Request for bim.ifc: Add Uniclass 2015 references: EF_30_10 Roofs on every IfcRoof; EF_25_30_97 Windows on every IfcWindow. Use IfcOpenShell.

First a look at what the model holds.

```python
import ifcopenshell

model = ifcopenshell.open("bim.ifc")
print(model.schema)
print("classifications:", [c.Name for c in model.by_type("IfcClassification")])
for ifc_class in ("IfcDoor", "IfcRoof", "IfcStair", "IfcWall", "IfcWindow"):
    print(ifc_class, len(model.by_type(ifc_class)))
```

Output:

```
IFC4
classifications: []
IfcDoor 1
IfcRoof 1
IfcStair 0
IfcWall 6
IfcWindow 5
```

```python
import ifcopenshell
import ifcopenshell.api.classification

model = ifcopenshell.open("bim.ifc")

system = ifcopenshell.api.classification.add_classification(model, classification="Uniclass 2015")

codes = {
    "IfcRoof": ("EF_30_10", "Roofs"),
    "IfcWindow": ("EF_25_30_97", "Windows"),
}
for ifc_class, (code, name) in codes.items():
    products = model.by_type(ifc_class)
    ifcopenshell.api.classification.add_reference(
        model, products=products, classification=system, identification=code, name=name
    )
    print(code, len(products))

model.write("bim_updated.ifc")
```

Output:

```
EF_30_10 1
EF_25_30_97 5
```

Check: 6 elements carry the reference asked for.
